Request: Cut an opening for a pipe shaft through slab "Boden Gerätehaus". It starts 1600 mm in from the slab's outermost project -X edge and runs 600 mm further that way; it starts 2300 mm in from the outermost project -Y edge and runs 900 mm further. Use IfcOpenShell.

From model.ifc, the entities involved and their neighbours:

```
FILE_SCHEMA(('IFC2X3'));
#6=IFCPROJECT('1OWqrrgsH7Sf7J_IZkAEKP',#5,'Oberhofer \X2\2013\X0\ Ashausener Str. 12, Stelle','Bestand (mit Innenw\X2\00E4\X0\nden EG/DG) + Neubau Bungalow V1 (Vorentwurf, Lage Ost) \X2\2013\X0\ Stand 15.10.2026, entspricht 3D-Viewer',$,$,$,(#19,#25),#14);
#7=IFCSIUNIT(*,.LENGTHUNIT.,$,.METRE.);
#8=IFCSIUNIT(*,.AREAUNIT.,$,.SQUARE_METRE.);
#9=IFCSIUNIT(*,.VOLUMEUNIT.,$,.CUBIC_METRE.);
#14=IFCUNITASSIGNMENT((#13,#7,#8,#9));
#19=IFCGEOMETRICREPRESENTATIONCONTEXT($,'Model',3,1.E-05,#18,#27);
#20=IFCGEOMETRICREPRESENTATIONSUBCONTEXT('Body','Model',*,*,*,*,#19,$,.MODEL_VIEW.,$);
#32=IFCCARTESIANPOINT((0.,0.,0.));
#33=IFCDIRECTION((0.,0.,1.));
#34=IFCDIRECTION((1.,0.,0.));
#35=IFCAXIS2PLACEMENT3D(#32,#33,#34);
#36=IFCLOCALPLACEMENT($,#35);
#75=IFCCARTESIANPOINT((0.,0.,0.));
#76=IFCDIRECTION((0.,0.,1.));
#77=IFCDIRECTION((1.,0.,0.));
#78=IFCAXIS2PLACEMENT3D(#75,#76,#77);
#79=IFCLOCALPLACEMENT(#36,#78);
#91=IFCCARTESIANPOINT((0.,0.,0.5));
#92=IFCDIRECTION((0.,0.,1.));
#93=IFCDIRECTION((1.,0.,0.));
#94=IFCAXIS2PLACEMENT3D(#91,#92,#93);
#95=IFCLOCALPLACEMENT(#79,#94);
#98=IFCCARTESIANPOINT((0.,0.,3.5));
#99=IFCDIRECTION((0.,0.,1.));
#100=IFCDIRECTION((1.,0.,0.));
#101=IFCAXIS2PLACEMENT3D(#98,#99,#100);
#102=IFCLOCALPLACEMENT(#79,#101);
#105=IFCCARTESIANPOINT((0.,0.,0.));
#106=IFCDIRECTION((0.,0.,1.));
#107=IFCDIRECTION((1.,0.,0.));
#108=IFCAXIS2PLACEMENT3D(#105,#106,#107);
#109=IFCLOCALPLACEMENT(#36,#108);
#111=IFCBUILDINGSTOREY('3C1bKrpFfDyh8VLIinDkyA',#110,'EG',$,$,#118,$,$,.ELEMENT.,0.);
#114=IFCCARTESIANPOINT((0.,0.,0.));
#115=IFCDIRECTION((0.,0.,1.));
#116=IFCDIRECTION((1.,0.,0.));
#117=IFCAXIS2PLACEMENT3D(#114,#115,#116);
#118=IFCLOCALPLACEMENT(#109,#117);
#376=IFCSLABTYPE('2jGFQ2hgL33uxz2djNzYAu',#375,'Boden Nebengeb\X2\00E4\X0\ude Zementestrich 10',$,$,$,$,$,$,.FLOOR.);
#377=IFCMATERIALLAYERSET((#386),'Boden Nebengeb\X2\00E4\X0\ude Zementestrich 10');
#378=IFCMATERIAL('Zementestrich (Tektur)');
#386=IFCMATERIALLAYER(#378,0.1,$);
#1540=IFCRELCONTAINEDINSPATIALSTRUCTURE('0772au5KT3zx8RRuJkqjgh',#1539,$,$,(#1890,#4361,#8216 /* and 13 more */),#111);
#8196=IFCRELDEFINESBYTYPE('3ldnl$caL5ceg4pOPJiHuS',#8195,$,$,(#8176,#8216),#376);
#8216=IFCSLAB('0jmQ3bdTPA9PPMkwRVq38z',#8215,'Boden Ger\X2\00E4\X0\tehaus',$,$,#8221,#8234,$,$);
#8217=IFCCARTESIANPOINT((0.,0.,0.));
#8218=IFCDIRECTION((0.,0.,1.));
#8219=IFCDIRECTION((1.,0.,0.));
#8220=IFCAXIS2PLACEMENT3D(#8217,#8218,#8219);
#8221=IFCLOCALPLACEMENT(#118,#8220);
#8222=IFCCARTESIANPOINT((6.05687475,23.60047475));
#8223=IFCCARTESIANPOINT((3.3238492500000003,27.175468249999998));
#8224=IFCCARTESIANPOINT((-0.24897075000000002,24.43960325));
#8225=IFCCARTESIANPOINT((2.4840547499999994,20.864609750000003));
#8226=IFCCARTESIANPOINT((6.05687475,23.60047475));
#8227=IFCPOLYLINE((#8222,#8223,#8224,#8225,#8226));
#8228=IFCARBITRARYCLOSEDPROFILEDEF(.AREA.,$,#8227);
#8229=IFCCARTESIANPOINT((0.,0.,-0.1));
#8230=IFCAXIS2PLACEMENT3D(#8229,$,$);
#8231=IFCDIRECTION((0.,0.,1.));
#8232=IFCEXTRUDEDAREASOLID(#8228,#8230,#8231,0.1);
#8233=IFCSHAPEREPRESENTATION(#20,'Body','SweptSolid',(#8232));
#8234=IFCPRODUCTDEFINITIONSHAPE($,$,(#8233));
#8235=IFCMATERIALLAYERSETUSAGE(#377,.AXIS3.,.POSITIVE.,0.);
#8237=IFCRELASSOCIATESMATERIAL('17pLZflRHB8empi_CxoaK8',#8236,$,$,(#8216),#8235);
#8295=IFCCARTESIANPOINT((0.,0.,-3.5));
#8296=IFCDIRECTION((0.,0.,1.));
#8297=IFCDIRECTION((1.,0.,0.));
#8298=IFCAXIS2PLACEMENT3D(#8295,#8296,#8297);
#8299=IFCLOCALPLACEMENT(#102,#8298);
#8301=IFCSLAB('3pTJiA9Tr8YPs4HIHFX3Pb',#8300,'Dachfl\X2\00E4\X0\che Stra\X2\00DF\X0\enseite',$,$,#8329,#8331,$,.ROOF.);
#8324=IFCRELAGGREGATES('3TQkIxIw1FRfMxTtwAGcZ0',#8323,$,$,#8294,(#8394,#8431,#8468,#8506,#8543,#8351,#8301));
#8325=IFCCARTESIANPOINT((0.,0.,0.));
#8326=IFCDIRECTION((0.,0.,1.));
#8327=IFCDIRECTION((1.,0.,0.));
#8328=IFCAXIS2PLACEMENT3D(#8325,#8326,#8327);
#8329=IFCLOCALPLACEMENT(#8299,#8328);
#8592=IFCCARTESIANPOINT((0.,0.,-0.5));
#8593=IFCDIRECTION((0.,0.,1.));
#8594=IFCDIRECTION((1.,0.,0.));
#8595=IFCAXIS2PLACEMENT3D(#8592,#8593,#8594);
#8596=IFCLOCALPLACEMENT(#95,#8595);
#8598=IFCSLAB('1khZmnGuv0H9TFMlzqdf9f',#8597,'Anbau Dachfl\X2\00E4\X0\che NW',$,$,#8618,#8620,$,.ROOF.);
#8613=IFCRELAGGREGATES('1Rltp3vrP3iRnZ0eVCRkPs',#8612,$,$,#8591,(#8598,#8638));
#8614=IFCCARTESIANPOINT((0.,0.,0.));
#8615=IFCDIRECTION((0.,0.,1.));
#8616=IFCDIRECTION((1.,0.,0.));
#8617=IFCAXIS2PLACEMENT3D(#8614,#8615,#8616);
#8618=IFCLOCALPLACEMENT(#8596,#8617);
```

```python
import numpy as np
import ifcopenshell
import ifcopenshell.api.feature
import ifcopenshell.api.geometry
import ifcopenshell.api.root
import ifcopenshell.geom
import ifcopenshell.util.placement
import ifcopenshell.util.representation
import ifcopenshell.util.shape
import ifcopenshell.util.unit

model = ifcopenshell.open("model.ifc")
unit_scale = ifcopenshell.util.unit.calculate_unit_scale(model)
settings = ifcopenshell.geom.settings()


def volume(element):
    """Net volume in cubic metres, openings subtracted."""
    shape = ifcopenshell.geom.create_shape(settings, element)
    return ifcopenshell.util.shape.get_volume(shape.geometry)


slab = model.by_id(8216)
before = volume(slab)

# Extent in the slab's own axes, in metres. The edges named are its -X and -Y sides.
slab_shape = ifcopenshell.geom.create_shape(settings, slab)
vertices = ifcopenshell.util.shape.get_vertices(slab_shape.geometry)
x_min, y_min, bottom = vertices.min(axis=0)
top = vertices[:, 2].max()

opening = ifcopenshell.api.root.create_entity(model, ifc_class="IfcOpeningElement", name="Pipe shaft opening")
context = ifcopenshell.util.representation.get_context(model, "Model", "Body", "MODEL_VIEW")
width, depth = 0.6, 0.9
outline = [(0.0, 0.0), (width, 0.0), (width, depth), (0.0, depth), (0.0, 0.0)]
# Overshoot both faces by 50 mm so the cut is clean.
shape = ifcopenshell.api.geometry.add_slab_representation(
    model, context=context, depth=top - bottom + 0.1, polyline=outline
)
ifcopenshell.api.geometry.assign_representation(model, product=opening, representation=shape)

matrix = ifcopenshell.util.placement.get_local_placement(slab.ObjectPlacement)
matrix[:, 3] = matrix @ np.append(np.array([x_min + 1.6, y_min + 2.3, bottom - 0.05]) / unit_scale, 1.0)
ifcopenshell.api.geometry.edit_object_placement(model, product=opening, matrix=matrix, is_si=False)
ifcopenshell.api.feature.add_feature(model, feature=opening, element=slab)

after = volume(slab)

print(f"slab volume {before:.3f} -> {after:.3f} m3")

model.write("model_v2.ifc")
```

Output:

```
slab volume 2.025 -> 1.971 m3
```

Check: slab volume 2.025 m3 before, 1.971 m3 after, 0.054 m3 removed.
